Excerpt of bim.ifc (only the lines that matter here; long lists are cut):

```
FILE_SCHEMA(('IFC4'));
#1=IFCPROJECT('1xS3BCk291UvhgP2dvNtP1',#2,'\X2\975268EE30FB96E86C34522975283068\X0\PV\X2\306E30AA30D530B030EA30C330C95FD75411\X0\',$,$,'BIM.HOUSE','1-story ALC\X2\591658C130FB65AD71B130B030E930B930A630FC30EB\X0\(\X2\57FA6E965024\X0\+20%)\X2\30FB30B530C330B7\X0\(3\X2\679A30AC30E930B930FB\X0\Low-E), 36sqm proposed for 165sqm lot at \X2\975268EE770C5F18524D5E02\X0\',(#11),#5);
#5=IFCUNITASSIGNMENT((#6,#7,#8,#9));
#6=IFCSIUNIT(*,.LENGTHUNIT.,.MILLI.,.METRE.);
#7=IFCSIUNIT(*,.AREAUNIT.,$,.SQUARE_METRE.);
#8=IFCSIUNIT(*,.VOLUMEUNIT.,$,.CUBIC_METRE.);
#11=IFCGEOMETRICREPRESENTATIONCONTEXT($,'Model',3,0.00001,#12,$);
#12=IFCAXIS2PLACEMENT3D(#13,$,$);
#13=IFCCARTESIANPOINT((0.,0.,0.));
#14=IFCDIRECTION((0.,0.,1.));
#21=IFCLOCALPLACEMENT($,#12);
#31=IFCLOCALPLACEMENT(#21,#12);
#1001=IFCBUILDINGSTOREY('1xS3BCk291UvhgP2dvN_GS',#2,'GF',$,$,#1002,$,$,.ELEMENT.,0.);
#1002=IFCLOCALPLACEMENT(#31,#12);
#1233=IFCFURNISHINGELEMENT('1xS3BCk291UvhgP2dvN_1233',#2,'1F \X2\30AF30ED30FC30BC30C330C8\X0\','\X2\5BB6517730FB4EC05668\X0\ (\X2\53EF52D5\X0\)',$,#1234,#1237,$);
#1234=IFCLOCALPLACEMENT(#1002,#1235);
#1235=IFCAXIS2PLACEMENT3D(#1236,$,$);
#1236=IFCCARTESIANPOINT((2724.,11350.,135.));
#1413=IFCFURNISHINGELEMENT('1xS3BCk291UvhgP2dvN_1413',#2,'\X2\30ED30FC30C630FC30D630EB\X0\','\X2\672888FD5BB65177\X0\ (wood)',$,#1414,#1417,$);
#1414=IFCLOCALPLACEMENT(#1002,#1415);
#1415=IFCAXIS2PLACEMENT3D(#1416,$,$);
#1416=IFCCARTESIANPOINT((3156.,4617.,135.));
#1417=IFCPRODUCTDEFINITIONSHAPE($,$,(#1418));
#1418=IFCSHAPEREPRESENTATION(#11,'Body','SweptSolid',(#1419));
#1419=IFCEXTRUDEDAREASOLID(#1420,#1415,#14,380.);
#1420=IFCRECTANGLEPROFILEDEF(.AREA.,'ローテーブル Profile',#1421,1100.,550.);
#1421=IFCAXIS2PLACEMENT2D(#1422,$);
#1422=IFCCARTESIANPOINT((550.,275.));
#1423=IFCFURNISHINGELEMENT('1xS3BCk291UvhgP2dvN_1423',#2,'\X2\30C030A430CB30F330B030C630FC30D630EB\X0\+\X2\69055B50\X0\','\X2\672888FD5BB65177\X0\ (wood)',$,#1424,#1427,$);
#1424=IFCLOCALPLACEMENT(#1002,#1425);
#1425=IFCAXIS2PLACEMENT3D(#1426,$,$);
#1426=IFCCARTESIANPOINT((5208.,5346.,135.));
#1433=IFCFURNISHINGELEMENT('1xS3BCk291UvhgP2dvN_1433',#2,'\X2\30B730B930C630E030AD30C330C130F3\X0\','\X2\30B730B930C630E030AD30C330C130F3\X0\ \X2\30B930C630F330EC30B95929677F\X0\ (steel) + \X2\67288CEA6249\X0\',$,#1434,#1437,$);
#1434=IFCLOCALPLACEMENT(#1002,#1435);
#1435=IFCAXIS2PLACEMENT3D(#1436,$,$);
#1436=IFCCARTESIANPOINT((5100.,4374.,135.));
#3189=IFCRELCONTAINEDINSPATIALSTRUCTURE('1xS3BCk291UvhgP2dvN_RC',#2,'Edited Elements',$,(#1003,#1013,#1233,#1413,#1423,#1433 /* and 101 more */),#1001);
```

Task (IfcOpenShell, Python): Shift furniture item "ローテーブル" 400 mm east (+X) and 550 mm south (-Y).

```python
import ifcopenshell
import ifcopenshell.api.geometry
import ifcopenshell.util.placement
import ifcopenshell.util.unit

model = ifcopenshell.open("bim.ifc")
unit_scale = ifcopenshell.util.unit.calculate_unit_scale(model)

item = model.by_guid("1xS3BCk291UvhgP2dvN_1413")
matrix = ifcopenshell.util.placement.get_local_placement(item.ObjectPlacement)
matrix[0, 3] += 0.4 / unit_scale
matrix[1, 3] -= 0.55 / unit_scale
ifcopenshell.api.geometry.edit_object_placement(model, product=item, matrix=matrix, is_si=False)

print(ifcopenshell.util.placement.get_local_placement(item.ObjectPlacement).round(3) + 0.0)

model.write("bim_rev.ifc")
```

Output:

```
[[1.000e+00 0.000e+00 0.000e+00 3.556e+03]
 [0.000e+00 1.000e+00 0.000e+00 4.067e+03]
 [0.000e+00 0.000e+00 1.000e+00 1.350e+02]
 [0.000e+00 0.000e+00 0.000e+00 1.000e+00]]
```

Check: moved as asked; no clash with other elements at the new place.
